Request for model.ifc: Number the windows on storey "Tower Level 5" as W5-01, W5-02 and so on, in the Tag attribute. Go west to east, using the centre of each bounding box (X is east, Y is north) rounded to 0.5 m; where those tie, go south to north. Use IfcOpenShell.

First a look at what the model holds.

```python
import ifcopenshell
import ifcopenshell.util.element
import ifcopenshell.util.placement

model = ifcopenshell.open("model.ifc")
print(model.schema)
storey = next(s for s in model.by_type("IfcBuildingStorey") if s.Name == "Tower Level 5")
windows = [e for e in ifcopenshell.util.element.get_decomposition(storey) if e.is_a("IfcWindow")]
for e in sorted(windows, key=lambda e: e.id()):
    origin = ifcopenshell.util.placement.get_local_placement(e.ObjectPlacement)[:3, 3]
    print(e.id(), e.Tag, e.Name, origin.round(2) + 0.0, sep=" | ")
```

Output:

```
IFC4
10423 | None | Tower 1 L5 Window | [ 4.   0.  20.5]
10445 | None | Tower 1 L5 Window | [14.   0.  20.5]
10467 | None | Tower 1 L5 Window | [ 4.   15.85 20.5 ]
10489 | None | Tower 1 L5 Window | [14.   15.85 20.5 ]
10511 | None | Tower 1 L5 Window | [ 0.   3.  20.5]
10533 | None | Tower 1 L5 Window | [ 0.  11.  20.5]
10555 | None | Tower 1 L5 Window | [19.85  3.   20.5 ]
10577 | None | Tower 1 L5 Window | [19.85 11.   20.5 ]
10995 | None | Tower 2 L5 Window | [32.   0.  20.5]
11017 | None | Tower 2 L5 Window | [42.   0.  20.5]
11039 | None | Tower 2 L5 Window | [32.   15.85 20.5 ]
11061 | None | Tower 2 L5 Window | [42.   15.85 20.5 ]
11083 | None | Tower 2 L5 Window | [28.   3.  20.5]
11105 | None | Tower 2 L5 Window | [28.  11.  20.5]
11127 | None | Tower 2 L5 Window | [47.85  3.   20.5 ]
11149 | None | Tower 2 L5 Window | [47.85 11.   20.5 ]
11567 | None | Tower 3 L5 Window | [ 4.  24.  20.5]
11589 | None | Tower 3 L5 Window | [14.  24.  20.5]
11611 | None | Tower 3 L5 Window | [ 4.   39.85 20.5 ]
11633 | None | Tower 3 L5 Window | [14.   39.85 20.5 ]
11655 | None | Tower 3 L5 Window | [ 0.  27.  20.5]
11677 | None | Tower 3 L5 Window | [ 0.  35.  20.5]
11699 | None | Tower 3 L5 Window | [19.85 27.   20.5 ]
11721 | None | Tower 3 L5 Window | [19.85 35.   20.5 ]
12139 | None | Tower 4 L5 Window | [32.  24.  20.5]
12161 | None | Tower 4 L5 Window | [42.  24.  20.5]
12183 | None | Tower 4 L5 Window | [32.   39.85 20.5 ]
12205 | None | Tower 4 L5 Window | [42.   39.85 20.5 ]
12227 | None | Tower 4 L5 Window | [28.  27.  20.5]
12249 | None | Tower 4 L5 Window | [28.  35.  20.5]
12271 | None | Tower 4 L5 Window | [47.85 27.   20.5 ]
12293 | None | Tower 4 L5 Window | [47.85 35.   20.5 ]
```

```python
import ifcopenshell
import ifcopenshell.geom
import ifcopenshell.util.element
import ifcopenshell.util.shape

model = ifcopenshell.open("model.ifc")
settings = ifcopenshell.geom.settings()
settings.set("use-world-coords", True)


def centre(element):
    shape = ifcopenshell.geom.create_shape(settings, element)
    return ifcopenshell.util.shape.get_bbox_centroid(shape.geometry)


storey = next(s for s in model.by_type("IfcBuildingStorey") if s.Name == "Tower Level 5")
windows = [e for e in ifcopenshell.util.element.get_decomposition(storey) if e.is_a("IfcWindow")]

# Insertion points can sit at a corner or the storey origin, so sort by the geometry (in metres).
centres = {e: centre(e) for e in windows}
windows.sort(key=lambda e: (round(centres[e][0] / 0.5), centres[e][1]))

for i, e in enumerate(windows, start=1):
    number = f"W5-{i:02d}"
    e.Tag = number
    print(e.id(), number)

model.write("model_edited.ifc")
```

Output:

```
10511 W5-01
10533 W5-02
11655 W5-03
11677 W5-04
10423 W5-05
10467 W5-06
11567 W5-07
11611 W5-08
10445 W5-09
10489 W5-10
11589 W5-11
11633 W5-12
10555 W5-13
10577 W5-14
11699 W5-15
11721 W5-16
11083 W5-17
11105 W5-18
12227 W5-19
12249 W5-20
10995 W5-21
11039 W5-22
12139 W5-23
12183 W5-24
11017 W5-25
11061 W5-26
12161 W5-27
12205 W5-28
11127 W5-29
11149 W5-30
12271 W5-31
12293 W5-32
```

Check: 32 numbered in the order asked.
